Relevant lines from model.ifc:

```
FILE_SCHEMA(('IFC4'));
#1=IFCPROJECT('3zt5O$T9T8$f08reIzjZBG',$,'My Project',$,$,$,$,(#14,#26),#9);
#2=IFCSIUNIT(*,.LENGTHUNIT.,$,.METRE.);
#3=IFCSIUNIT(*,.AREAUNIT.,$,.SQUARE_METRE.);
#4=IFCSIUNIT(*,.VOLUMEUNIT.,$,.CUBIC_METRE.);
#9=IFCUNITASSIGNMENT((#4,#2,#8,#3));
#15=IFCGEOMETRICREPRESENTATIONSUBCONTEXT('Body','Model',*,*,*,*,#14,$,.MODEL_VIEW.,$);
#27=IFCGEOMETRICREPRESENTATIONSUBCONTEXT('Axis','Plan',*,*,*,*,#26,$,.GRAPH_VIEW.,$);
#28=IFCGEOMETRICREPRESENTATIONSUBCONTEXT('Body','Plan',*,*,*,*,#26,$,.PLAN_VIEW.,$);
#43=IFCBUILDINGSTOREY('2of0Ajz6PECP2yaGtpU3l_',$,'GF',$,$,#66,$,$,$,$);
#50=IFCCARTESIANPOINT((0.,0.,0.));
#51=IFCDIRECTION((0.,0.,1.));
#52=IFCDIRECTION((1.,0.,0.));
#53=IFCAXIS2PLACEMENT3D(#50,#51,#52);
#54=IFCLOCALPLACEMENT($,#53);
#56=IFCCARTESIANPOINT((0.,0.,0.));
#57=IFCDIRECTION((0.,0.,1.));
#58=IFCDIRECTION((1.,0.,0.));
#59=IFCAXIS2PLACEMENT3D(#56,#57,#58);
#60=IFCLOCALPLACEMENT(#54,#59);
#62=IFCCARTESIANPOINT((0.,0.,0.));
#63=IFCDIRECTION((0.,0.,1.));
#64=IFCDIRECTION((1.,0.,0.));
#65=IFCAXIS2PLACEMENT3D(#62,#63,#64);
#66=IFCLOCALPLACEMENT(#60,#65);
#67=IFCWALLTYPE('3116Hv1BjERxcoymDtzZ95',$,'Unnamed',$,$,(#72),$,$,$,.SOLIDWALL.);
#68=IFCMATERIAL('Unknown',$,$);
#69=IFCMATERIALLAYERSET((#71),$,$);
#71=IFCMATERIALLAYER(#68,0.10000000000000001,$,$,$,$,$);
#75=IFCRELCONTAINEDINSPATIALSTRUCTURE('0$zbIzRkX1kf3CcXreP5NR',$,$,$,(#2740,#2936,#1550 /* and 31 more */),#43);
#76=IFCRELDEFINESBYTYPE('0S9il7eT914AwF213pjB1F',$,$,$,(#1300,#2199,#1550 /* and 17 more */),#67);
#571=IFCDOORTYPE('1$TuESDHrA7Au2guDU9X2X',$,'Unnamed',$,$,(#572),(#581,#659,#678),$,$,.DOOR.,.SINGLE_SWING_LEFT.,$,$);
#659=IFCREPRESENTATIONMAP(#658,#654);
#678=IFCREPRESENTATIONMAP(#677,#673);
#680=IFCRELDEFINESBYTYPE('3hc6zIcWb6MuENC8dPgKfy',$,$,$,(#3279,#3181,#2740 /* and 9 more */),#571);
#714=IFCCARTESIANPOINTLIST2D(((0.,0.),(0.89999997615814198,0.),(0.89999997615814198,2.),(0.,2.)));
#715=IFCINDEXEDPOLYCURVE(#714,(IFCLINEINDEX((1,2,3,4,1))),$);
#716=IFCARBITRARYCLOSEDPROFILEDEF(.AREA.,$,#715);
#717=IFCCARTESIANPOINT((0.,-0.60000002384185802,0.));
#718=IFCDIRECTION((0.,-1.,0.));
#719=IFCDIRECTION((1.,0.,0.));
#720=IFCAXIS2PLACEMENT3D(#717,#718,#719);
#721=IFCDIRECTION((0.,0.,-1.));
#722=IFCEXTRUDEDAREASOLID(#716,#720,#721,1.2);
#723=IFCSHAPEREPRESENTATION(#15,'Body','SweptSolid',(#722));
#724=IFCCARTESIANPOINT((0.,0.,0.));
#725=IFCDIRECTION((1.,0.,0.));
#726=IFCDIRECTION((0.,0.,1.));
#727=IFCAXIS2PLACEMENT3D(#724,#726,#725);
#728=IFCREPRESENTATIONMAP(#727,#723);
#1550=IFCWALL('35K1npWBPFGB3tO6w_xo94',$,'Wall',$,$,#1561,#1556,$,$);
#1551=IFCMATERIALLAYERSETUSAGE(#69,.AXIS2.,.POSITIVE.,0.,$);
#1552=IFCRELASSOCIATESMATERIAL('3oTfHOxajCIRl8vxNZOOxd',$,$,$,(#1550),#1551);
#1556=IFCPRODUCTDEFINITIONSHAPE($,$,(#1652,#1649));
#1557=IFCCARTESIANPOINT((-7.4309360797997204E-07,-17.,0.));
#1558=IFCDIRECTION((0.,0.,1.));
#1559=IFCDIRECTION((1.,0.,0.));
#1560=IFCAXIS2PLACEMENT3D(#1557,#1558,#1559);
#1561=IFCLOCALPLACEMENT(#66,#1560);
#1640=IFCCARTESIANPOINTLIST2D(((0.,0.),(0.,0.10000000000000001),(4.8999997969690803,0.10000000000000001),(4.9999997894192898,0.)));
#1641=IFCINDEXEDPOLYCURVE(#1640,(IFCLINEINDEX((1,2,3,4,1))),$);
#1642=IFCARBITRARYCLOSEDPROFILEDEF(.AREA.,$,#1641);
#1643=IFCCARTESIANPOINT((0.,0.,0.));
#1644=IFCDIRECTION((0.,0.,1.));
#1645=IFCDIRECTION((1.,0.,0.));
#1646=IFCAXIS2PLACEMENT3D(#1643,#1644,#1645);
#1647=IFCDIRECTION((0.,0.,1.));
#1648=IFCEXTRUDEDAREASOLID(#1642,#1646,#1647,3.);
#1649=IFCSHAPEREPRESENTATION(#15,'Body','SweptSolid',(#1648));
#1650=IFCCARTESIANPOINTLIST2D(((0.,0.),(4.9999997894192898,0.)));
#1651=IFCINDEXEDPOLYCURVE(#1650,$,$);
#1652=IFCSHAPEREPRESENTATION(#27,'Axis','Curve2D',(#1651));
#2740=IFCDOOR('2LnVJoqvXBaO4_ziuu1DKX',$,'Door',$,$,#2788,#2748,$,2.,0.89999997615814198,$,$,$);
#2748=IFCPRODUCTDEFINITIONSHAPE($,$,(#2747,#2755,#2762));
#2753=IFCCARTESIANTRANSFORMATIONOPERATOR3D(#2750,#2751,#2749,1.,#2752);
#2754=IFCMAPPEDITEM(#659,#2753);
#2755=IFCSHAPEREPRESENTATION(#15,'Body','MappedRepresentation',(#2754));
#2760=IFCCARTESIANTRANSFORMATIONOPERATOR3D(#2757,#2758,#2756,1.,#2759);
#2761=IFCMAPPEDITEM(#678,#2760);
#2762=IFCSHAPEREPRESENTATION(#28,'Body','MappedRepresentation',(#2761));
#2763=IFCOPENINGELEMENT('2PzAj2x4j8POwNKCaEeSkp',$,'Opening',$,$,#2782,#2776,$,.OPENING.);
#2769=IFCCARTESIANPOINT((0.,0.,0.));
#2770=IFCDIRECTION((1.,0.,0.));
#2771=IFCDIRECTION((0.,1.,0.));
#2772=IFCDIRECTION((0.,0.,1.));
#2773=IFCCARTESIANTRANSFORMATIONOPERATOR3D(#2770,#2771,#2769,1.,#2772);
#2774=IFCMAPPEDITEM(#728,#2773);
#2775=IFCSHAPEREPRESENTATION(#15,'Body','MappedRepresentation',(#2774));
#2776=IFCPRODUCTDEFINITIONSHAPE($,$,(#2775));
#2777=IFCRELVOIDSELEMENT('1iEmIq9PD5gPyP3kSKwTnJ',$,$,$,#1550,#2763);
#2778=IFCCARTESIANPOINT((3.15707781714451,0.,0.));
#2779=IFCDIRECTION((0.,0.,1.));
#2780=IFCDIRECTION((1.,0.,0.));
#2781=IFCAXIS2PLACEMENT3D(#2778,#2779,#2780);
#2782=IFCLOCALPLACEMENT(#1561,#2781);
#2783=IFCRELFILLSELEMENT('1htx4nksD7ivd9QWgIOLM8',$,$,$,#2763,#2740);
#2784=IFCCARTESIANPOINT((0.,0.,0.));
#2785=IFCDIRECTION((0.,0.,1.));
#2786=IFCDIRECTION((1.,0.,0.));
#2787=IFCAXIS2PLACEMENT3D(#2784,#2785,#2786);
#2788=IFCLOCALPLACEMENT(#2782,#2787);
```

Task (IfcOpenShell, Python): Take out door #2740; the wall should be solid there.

```python
import ifcopenshell
import ifcopenshell.api.feature
import ifcopenshell.api.root
import ifcopenshell.geom
import ifcopenshell.util.shape

model = ifcopenshell.open("model.ifc")
settings = ifcopenshell.geom.settings()


def volume(element):
    """Net volume in cubic metres, openings subtracted."""
    shape = ifcopenshell.geom.create_shape(settings, element)
    return ifcopenshell.util.shape.get_volume(shape.geometry)


door = model.by_guid("2LnVJoqvXBaO4_ziuu1DKX")
opening = door.FillsVoids[0].RelatingOpeningElement
wall = opening.VoidsElements[0].RelatingBuildingElement
before = volume(wall)

ifcopenshell.api.root.remove_product(model, product=door)
ifcopenshell.api.feature.remove_feature(model, feature=opening)

after = volume(wall)

print(f"wall volume {before:.3f} -> {after:.3f} m3")

model.write("model_edited.ifc")
```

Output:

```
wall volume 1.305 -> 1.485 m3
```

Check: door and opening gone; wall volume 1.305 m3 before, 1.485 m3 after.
